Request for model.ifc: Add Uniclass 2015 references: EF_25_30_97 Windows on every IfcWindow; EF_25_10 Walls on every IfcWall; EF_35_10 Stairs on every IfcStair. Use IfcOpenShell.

First a look at what the model holds.

```python
import ifcopenshell

model = ifcopenshell.open("model.ifc")
print(model.schema)
print("classifications:", [c.Name for c in model.by_type("IfcClassification")])
for ifc_class in ("IfcDoor", "IfcRoof", "IfcStair", "IfcWall", "IfcWindow"):
    print(ifc_class, len(model.by_type(ifc_class)))
```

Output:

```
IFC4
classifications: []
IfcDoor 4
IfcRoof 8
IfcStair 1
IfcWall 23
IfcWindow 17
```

```python
import ifcopenshell
import ifcopenshell.api.classification

model = ifcopenshell.open("model.ifc")

system = ifcopenshell.api.classification.add_classification(model, classification="Uniclass 2015")

codes = {
    "IfcWindow": ("EF_25_30_97", "Windows"),
    "IfcWall": ("EF_25_10", "Walls"),
    "IfcStair": ("EF_35_10", "Stairs"),
}
for ifc_class, (code, name) in codes.items():
    products = model.by_type(ifc_class)
    ifcopenshell.api.classification.add_reference(
        model, products=products, classification=system, identification=code, name=name
    )
    print(code, len(products))

model.write("model-out.ifc")
```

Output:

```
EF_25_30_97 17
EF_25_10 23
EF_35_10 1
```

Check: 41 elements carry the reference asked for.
